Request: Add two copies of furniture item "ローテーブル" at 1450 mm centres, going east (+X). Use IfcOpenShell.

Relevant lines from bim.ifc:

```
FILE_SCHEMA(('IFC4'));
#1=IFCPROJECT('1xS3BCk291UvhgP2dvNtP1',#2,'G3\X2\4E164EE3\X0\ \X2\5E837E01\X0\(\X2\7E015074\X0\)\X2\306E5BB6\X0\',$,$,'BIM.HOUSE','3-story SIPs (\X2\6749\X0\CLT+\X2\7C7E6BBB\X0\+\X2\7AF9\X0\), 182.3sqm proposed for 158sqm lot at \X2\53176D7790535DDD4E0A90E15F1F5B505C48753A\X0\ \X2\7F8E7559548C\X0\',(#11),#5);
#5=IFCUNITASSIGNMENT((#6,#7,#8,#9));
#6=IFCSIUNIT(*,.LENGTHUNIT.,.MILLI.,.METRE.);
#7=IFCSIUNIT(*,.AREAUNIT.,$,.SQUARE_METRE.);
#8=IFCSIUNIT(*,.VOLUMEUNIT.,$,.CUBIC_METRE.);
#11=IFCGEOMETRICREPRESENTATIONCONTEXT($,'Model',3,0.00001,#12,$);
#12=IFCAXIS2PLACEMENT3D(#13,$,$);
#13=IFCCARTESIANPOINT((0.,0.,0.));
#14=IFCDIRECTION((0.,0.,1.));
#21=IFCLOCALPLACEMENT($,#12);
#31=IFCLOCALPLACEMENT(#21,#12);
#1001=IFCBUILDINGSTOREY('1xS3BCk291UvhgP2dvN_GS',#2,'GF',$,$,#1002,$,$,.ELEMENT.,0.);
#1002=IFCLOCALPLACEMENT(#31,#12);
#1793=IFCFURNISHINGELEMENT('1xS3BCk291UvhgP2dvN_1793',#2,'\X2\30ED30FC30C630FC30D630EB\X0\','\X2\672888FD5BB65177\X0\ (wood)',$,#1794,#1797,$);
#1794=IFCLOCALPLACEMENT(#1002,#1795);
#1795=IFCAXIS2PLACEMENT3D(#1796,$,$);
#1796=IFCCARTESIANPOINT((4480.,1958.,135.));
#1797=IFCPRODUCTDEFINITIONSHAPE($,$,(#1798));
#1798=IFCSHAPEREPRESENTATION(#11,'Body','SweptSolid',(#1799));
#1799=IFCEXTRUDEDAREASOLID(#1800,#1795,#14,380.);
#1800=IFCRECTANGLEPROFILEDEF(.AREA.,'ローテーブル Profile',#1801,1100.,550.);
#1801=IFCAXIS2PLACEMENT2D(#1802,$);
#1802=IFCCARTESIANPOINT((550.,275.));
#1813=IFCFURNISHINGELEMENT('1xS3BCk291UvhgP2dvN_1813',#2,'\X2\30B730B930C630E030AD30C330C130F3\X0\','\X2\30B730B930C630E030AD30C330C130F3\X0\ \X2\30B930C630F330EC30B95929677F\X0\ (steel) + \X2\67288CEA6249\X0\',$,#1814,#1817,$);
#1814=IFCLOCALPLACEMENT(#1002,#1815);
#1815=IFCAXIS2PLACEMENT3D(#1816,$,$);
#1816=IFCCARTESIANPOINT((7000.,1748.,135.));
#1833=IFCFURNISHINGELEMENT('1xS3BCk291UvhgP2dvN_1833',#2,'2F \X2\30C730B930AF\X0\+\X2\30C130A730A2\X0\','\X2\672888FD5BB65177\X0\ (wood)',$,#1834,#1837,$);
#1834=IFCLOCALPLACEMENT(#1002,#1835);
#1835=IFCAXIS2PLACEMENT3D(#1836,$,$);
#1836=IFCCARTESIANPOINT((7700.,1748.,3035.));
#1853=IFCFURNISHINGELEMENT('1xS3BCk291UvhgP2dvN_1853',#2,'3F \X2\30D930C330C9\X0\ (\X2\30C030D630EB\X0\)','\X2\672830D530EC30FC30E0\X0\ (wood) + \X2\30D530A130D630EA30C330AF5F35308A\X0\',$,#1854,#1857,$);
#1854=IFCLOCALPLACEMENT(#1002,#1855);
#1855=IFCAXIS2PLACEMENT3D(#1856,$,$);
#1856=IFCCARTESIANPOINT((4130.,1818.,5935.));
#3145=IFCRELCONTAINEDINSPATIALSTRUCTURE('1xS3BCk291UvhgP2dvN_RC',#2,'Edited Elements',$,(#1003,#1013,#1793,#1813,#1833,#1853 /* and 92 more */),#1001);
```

```python
import numpy as np
import ifcopenshell
import ifcopenshell.api.geometry
import ifcopenshell.api.root
import ifcopenshell.util.element
import ifcopenshell.util.placement
import ifcopenshell.util.unit

model = ifcopenshell.open("bim.ifc")
unit_scale = ifcopenshell.util.unit.calculate_unit_scale(model)


def reuse_history(source, copy):
    """copy_class also copies each property set's owner history, people and application; keep the originals."""
    for rel in copy.IsDefinedBy:
        if rel.is_a("IfcRelDefinesByProperties") and (history := rel.RelatingPropertyDefinition.OwnerHistory):
            rel.RelatingPropertyDefinition.OwnerHistory = source.OwnerHistory
            ifcopenshell.util.element.remove_deep2(model, history)


source = model.by_guid("1xS3BCk291UvhgP2dvN_1793")
base = ifcopenshell.util.placement.get_local_placement(source.ObjectPlacement)
step = np.array([1.0, 0.0, 0.0]) * 1.45 / unit_scale

for i in range(1, 3):
    copy = ifcopenshell.api.root.copy_class(model, product=source)
    copy.Representation = ifcopenshell.util.element.copy_deep(
        model, source.Representation, exclude=["IfcGeometricRepresentationContext", "IfcRepresentationMap"]
    )
    reuse_history(source, copy)
    matrix = base.copy()
    matrix[:3, 3] += i * step
    print("added at", matrix[:3, 3].round(3) + 0.0)
    ifcopenshell.api.geometry.edit_object_placement(model, product=copy, matrix=matrix, is_si=False)

model.write("bim_updated.ifc")
```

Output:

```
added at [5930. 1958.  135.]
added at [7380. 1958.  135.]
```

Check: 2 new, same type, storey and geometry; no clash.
